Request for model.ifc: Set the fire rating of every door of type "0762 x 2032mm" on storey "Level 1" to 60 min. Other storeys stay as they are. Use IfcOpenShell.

First a look at what the model holds.

```python
import ifcopenshell
import ifcopenshell.util.element

model = ifcopenshell.open("model.ifc")
print(model.schema)
storey = next(s for s in model.by_type("IfcBuildingStorey") if s.Name == "Level 1")
doors = [e for e in ifcopenshell.util.element.get_decomposition(storey) if e.is_a("IfcDoor")]
seen = {}
for e in doors:
    element_type = ifcopenshell.util.element.get_type(e)
    key = (element_type.Name if element_type != e and element_type else None, ifcopenshell.util.element.get_pset(e, "Pset_DoorCommon", "FireRating"))
    seen[key] = seen.get(key, 0) + 1
for (name, value), count in sorted(seen.items(), key=str):
    print(count, "x", name, "|", value)
```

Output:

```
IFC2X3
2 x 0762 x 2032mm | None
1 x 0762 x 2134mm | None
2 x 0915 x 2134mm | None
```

```python
import ifcopenshell
import ifcopenshell.api.pset
import ifcopenshell.util.element

model = ifcopenshell.open("model.ifc")

storey = next(s for s in model.by_type("IfcBuildingStorey") if s.Name == "Level 1")
doors = [e for e in ifcopenshell.util.element.get_decomposition(storey) if e.is_a("IfcDoor")]

count = 0
for e in doors:
    element_type = ifcopenshell.util.element.get_type(e)
    if element_type in (None, e) or element_type.Name != "0762 x 2032mm":
        continue
    # add_pset returns the element's existing set when there is one.
    pset = ifcopenshell.api.pset.add_pset(model, product=e, name="Pset_DoorCommon")
    ifcopenshell.api.pset.edit_pset(model, pset=pset, properties={"FireRating": "60 min"})
    count += 1

print(count, "doors updated")

model.write("model_rev.ifc")
```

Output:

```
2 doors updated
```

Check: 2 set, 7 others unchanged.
